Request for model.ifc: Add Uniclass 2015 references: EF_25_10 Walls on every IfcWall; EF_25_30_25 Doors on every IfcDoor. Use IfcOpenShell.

First a look at what the model holds.

```python
import ifcopenshell

model = ifcopenshell.open("model.ifc")
print(model.schema)
print("classifications:", [c.Name for c in model.by_type("IfcClassification")])
for ifc_class in ("IfcDoor", "IfcRoof", "IfcStair", "IfcWall", "IfcWindow"):
    print(ifc_class, len(model.by_type(ifc_class)))
```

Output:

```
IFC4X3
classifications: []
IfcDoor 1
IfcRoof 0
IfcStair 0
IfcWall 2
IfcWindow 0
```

```python
import ifcopenshell
import ifcopenshell.api.classification

model = ifcopenshell.open("model.ifc")

system = ifcopenshell.api.classification.add_classification(model, classification="Uniclass 2015")

codes = {
    "IfcWall": ("EF_25_10", "Walls"),
    "IfcDoor": ("EF_25_30_25", "Doors"),
}
for ifc_class, (code, name) in codes.items():
    products = model.by_type(ifc_class)
    ifcopenshell.api.classification.add_reference(
        model, products=products, classification=system, identification=code, name=name
    )
    print(code, len(products))

model.write("model-out.ifc")
```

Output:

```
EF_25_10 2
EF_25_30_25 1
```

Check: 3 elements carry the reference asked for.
